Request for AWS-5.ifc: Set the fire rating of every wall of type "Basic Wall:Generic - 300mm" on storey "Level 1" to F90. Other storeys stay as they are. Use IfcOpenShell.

First a look at what the model holds.

```python
import ifcopenshell
import ifcopenshell.util.element

model = ifcopenshell.open("AWS-5.ifc")
print(model.schema)
storey = next(s for s in model.by_type("IfcBuildingStorey") if s.Name == "Level 1")
walls = [e for e in ifcopenshell.util.element.get_decomposition(storey) if e.is_a("IfcWall")]
seen = {}
for e in walls:
    element_type = ifcopenshell.util.element.get_type(e)
    key = (element_type.Name if element_type != e and element_type else None, ifcopenshell.util.element.get_pset(e, "Pset_WallCommon", "FireRating"))
    seen[key] = seen.get(key, 0) + 1
for (name, value), count in sorted(seen.items(), key=str):
    print(count, "x", name, "|", value)
```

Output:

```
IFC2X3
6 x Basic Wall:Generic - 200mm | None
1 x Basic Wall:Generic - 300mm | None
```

```python
import ifcopenshell
import ifcopenshell.api.pset
import ifcopenshell.util.element

model = ifcopenshell.open("AWS-5.ifc")

storey = next(s for s in model.by_type("IfcBuildingStorey") if s.Name == "Level 1")
walls = [e for e in ifcopenshell.util.element.get_decomposition(storey) if e.is_a("IfcWall")]

count = 0
for e in walls:
    element_type = ifcopenshell.util.element.get_type(e)
    if element_type in (None, e) or element_type.Name != "Basic Wall:Generic - 300mm":
        continue
    # add_pset returns the element's existing set when there is one.
    pset = ifcopenshell.api.pset.add_pset(model, product=e, name="Pset_WallCommon")
    ifcopenshell.api.pset.edit_pset(model, pset=pset, properties={"FireRating": "F90"})
    count += 1

print(count, "walls updated")

model.write("AWS-5_edited.ifc")
```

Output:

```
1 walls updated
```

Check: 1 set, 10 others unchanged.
